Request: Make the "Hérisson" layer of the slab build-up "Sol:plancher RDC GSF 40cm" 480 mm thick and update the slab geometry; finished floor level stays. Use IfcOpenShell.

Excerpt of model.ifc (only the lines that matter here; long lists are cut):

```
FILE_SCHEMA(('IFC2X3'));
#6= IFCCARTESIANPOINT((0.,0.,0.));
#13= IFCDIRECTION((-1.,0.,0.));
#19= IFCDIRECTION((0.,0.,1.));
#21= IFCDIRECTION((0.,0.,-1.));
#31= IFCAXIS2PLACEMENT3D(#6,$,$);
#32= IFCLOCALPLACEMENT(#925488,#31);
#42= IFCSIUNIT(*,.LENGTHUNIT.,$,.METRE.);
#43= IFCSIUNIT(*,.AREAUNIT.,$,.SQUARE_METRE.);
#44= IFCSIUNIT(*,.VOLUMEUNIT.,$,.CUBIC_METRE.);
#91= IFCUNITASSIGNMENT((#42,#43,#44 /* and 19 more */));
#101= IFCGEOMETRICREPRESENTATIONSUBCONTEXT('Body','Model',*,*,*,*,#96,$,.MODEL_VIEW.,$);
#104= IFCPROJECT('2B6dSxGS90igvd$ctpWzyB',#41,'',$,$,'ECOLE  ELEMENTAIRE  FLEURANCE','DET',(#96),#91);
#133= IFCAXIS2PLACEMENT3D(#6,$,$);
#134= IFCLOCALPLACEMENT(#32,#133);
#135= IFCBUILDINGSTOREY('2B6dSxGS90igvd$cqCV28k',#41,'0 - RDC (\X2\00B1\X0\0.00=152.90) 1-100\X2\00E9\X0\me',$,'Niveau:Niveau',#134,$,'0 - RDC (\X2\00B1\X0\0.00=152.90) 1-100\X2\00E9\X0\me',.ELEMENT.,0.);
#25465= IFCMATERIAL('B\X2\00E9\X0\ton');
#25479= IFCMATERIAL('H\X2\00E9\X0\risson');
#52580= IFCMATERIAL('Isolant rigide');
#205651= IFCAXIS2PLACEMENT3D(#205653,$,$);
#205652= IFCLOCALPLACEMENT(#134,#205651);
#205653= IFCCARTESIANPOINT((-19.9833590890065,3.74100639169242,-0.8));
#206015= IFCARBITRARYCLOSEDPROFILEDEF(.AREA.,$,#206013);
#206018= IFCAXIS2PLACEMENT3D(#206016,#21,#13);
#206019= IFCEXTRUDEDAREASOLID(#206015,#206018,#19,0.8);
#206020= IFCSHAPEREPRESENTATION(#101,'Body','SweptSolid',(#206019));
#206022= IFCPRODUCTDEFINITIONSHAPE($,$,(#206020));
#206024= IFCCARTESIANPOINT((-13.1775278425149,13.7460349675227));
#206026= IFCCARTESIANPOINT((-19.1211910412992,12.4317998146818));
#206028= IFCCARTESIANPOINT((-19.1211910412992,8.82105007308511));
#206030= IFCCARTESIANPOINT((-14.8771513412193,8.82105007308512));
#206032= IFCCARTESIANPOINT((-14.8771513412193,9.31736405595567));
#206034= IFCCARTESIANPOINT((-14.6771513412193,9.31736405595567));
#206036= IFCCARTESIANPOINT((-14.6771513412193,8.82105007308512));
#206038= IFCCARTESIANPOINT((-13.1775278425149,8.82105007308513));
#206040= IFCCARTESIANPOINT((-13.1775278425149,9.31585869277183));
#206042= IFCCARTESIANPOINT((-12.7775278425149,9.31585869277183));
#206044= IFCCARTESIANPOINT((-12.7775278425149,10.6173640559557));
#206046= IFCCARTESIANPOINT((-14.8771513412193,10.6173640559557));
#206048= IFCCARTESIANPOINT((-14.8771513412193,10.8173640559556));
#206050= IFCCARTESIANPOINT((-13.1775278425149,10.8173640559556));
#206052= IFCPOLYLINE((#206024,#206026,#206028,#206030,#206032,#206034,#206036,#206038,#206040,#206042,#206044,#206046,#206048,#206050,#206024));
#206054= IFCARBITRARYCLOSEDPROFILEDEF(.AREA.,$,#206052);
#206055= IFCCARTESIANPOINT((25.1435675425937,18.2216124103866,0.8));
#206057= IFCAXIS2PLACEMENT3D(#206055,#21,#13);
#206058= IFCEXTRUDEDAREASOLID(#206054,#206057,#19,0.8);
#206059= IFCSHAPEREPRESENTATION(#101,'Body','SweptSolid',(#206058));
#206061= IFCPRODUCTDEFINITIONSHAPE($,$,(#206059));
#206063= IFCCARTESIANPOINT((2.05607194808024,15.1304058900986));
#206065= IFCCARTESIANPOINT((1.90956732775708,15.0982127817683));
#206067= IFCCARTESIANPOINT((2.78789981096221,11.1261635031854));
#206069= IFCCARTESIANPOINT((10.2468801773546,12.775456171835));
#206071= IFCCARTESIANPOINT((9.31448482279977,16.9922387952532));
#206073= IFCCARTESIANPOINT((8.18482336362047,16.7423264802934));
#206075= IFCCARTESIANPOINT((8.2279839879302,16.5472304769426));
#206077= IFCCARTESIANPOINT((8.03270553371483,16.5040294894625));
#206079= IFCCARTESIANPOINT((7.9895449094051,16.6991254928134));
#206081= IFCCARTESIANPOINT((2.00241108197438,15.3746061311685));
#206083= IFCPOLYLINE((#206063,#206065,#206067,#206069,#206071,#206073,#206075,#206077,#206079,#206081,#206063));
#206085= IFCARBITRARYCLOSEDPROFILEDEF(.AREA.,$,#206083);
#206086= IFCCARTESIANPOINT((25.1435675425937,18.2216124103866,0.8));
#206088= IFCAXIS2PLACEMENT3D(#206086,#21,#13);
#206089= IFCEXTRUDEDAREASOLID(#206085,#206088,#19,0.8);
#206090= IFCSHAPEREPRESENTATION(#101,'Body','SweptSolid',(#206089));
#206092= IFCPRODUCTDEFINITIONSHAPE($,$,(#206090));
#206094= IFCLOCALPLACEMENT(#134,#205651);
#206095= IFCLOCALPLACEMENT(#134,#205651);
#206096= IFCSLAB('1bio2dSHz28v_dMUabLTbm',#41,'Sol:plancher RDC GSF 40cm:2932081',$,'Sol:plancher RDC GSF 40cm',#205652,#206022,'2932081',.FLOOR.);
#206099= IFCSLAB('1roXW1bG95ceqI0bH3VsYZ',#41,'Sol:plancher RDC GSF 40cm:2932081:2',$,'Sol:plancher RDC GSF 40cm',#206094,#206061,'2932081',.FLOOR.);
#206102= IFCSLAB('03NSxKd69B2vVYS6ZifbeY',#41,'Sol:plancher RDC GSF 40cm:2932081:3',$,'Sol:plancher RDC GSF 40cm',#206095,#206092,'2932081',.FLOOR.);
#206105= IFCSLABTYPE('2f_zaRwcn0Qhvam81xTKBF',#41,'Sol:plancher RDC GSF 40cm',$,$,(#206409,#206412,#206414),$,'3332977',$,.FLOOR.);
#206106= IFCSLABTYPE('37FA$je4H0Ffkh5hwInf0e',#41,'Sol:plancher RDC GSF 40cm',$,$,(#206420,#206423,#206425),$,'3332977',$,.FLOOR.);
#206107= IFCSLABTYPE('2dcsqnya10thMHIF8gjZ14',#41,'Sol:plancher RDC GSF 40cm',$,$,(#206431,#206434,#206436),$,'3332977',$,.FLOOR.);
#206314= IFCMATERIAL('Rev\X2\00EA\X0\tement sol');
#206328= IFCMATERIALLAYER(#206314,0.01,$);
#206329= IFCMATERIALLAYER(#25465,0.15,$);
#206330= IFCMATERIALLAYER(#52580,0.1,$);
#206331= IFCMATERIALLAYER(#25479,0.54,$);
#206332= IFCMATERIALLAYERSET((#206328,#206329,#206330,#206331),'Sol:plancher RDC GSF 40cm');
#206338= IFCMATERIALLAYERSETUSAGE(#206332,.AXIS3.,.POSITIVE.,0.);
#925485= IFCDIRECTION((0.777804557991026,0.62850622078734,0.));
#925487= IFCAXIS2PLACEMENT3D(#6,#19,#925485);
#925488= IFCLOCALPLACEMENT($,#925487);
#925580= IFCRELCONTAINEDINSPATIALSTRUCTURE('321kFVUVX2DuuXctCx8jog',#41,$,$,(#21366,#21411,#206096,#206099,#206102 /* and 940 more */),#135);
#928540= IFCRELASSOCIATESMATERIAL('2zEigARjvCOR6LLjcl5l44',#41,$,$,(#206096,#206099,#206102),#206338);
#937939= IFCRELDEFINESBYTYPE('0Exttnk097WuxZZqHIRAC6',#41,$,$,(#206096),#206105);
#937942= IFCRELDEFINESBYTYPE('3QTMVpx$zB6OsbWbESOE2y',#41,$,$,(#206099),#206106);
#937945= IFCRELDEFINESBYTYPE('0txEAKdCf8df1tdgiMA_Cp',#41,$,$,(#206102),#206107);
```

```python
import ifcopenshell
import ifcopenshell.util.element
import ifcopenshell.util.representation

model = ifcopenshell.open("model.ifc")

layer_set = model.by_id(206332)
layer = next(l for l in layer_set.MaterialLayers if l.Material and l.Material.Name == "Hérisson")
change = 0.48 - layer.LayerThickness
layer.LayerThickness += change

# The layer set is shared, so every slab that uses it gets the new thickness.
slabs = [e for e in ifcopenshell.util.element.get_elements_by_material(model, layer_set) if e.is_a("IfcSlab")]
for slab in sorted(slabs, key=lambda e: e.id()):
    body = ifcopenshell.util.representation.get_representation(slab, "Model", "Body")
    solid = body.Items[0]
    old_depth = solid.Depth
    solid.Depth += change
    print(slab.id(), f"{old_depth:g} -> {solid.Depth:g}")

# The layers are counted up from the underside, which has moved.
for usage in {ifcopenshell.util.element.get_material(slab) for slab in slabs}:
    usage.OffsetFromReferenceLine -= change

model.write("model_edited.ifc")
```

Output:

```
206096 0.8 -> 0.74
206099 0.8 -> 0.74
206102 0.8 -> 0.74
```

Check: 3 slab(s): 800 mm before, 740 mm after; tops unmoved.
